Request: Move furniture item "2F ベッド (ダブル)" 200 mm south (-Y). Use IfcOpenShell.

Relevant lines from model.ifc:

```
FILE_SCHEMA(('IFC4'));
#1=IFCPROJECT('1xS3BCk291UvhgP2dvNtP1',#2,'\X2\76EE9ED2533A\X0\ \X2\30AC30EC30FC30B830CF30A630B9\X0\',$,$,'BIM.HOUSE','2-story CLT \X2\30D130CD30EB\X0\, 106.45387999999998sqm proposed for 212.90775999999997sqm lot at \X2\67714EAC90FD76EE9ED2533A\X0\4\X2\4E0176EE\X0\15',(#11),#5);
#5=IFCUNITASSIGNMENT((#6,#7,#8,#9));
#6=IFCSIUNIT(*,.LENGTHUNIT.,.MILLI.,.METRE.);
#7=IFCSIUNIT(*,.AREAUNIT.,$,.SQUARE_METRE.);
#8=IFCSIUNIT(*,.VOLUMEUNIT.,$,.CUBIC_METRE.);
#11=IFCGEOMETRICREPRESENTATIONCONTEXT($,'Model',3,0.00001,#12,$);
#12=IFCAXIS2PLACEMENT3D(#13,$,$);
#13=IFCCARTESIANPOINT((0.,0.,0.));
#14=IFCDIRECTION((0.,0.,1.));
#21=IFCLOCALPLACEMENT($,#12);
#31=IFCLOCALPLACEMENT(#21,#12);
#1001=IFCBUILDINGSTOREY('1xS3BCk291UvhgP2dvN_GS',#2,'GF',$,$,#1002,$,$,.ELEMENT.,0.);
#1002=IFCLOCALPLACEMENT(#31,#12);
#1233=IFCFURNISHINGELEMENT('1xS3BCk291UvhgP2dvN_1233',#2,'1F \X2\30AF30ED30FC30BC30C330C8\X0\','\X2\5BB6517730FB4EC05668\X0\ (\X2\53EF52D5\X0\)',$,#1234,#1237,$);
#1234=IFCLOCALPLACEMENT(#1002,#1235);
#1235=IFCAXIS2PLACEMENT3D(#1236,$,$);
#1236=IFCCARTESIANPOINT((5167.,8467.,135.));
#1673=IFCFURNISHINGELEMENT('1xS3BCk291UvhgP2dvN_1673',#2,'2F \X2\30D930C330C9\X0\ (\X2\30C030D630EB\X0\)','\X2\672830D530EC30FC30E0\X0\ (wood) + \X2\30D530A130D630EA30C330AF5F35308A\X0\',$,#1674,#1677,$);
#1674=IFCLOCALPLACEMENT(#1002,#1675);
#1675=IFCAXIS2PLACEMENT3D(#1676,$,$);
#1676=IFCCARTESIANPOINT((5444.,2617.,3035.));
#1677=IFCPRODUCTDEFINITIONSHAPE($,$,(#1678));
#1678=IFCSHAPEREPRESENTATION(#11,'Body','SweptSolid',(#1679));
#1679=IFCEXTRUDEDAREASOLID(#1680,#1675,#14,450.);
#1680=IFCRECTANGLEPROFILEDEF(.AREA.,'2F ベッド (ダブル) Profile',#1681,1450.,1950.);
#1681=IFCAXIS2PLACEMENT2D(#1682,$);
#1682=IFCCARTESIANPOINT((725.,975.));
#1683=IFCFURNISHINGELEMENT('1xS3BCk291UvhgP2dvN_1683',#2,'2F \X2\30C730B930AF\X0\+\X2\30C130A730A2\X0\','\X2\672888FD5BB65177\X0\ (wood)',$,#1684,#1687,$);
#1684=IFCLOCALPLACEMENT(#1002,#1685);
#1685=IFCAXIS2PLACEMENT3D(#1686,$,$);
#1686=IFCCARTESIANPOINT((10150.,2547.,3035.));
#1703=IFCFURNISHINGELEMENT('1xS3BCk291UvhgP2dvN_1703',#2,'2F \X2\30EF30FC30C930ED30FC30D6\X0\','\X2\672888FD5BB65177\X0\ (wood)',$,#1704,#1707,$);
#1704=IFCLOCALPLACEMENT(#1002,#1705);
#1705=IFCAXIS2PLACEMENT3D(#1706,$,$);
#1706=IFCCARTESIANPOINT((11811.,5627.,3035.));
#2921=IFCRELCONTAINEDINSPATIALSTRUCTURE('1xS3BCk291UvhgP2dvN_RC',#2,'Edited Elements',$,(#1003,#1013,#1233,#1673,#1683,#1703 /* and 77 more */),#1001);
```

```python
import ifcopenshell
import ifcopenshell.api.geometry
import ifcopenshell.util.placement

model = ifcopenshell.open("model.ifc")

item = model.by_id(1673)
matrix = ifcopenshell.util.placement.get_local_placement(item.ObjectPlacement)
matrix[1, 3] -= 200.0
ifcopenshell.api.geometry.edit_object_placement(model, product=item, matrix=matrix, is_si=False)

print(ifcopenshell.util.placement.get_local_placement(item.ObjectPlacement).round(3) + 0.0)

model.write("model_rev.ifc")
```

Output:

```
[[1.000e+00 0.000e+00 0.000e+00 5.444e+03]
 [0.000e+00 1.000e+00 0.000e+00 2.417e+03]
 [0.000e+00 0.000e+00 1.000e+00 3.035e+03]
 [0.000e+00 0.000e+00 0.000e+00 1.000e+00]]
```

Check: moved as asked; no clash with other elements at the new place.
